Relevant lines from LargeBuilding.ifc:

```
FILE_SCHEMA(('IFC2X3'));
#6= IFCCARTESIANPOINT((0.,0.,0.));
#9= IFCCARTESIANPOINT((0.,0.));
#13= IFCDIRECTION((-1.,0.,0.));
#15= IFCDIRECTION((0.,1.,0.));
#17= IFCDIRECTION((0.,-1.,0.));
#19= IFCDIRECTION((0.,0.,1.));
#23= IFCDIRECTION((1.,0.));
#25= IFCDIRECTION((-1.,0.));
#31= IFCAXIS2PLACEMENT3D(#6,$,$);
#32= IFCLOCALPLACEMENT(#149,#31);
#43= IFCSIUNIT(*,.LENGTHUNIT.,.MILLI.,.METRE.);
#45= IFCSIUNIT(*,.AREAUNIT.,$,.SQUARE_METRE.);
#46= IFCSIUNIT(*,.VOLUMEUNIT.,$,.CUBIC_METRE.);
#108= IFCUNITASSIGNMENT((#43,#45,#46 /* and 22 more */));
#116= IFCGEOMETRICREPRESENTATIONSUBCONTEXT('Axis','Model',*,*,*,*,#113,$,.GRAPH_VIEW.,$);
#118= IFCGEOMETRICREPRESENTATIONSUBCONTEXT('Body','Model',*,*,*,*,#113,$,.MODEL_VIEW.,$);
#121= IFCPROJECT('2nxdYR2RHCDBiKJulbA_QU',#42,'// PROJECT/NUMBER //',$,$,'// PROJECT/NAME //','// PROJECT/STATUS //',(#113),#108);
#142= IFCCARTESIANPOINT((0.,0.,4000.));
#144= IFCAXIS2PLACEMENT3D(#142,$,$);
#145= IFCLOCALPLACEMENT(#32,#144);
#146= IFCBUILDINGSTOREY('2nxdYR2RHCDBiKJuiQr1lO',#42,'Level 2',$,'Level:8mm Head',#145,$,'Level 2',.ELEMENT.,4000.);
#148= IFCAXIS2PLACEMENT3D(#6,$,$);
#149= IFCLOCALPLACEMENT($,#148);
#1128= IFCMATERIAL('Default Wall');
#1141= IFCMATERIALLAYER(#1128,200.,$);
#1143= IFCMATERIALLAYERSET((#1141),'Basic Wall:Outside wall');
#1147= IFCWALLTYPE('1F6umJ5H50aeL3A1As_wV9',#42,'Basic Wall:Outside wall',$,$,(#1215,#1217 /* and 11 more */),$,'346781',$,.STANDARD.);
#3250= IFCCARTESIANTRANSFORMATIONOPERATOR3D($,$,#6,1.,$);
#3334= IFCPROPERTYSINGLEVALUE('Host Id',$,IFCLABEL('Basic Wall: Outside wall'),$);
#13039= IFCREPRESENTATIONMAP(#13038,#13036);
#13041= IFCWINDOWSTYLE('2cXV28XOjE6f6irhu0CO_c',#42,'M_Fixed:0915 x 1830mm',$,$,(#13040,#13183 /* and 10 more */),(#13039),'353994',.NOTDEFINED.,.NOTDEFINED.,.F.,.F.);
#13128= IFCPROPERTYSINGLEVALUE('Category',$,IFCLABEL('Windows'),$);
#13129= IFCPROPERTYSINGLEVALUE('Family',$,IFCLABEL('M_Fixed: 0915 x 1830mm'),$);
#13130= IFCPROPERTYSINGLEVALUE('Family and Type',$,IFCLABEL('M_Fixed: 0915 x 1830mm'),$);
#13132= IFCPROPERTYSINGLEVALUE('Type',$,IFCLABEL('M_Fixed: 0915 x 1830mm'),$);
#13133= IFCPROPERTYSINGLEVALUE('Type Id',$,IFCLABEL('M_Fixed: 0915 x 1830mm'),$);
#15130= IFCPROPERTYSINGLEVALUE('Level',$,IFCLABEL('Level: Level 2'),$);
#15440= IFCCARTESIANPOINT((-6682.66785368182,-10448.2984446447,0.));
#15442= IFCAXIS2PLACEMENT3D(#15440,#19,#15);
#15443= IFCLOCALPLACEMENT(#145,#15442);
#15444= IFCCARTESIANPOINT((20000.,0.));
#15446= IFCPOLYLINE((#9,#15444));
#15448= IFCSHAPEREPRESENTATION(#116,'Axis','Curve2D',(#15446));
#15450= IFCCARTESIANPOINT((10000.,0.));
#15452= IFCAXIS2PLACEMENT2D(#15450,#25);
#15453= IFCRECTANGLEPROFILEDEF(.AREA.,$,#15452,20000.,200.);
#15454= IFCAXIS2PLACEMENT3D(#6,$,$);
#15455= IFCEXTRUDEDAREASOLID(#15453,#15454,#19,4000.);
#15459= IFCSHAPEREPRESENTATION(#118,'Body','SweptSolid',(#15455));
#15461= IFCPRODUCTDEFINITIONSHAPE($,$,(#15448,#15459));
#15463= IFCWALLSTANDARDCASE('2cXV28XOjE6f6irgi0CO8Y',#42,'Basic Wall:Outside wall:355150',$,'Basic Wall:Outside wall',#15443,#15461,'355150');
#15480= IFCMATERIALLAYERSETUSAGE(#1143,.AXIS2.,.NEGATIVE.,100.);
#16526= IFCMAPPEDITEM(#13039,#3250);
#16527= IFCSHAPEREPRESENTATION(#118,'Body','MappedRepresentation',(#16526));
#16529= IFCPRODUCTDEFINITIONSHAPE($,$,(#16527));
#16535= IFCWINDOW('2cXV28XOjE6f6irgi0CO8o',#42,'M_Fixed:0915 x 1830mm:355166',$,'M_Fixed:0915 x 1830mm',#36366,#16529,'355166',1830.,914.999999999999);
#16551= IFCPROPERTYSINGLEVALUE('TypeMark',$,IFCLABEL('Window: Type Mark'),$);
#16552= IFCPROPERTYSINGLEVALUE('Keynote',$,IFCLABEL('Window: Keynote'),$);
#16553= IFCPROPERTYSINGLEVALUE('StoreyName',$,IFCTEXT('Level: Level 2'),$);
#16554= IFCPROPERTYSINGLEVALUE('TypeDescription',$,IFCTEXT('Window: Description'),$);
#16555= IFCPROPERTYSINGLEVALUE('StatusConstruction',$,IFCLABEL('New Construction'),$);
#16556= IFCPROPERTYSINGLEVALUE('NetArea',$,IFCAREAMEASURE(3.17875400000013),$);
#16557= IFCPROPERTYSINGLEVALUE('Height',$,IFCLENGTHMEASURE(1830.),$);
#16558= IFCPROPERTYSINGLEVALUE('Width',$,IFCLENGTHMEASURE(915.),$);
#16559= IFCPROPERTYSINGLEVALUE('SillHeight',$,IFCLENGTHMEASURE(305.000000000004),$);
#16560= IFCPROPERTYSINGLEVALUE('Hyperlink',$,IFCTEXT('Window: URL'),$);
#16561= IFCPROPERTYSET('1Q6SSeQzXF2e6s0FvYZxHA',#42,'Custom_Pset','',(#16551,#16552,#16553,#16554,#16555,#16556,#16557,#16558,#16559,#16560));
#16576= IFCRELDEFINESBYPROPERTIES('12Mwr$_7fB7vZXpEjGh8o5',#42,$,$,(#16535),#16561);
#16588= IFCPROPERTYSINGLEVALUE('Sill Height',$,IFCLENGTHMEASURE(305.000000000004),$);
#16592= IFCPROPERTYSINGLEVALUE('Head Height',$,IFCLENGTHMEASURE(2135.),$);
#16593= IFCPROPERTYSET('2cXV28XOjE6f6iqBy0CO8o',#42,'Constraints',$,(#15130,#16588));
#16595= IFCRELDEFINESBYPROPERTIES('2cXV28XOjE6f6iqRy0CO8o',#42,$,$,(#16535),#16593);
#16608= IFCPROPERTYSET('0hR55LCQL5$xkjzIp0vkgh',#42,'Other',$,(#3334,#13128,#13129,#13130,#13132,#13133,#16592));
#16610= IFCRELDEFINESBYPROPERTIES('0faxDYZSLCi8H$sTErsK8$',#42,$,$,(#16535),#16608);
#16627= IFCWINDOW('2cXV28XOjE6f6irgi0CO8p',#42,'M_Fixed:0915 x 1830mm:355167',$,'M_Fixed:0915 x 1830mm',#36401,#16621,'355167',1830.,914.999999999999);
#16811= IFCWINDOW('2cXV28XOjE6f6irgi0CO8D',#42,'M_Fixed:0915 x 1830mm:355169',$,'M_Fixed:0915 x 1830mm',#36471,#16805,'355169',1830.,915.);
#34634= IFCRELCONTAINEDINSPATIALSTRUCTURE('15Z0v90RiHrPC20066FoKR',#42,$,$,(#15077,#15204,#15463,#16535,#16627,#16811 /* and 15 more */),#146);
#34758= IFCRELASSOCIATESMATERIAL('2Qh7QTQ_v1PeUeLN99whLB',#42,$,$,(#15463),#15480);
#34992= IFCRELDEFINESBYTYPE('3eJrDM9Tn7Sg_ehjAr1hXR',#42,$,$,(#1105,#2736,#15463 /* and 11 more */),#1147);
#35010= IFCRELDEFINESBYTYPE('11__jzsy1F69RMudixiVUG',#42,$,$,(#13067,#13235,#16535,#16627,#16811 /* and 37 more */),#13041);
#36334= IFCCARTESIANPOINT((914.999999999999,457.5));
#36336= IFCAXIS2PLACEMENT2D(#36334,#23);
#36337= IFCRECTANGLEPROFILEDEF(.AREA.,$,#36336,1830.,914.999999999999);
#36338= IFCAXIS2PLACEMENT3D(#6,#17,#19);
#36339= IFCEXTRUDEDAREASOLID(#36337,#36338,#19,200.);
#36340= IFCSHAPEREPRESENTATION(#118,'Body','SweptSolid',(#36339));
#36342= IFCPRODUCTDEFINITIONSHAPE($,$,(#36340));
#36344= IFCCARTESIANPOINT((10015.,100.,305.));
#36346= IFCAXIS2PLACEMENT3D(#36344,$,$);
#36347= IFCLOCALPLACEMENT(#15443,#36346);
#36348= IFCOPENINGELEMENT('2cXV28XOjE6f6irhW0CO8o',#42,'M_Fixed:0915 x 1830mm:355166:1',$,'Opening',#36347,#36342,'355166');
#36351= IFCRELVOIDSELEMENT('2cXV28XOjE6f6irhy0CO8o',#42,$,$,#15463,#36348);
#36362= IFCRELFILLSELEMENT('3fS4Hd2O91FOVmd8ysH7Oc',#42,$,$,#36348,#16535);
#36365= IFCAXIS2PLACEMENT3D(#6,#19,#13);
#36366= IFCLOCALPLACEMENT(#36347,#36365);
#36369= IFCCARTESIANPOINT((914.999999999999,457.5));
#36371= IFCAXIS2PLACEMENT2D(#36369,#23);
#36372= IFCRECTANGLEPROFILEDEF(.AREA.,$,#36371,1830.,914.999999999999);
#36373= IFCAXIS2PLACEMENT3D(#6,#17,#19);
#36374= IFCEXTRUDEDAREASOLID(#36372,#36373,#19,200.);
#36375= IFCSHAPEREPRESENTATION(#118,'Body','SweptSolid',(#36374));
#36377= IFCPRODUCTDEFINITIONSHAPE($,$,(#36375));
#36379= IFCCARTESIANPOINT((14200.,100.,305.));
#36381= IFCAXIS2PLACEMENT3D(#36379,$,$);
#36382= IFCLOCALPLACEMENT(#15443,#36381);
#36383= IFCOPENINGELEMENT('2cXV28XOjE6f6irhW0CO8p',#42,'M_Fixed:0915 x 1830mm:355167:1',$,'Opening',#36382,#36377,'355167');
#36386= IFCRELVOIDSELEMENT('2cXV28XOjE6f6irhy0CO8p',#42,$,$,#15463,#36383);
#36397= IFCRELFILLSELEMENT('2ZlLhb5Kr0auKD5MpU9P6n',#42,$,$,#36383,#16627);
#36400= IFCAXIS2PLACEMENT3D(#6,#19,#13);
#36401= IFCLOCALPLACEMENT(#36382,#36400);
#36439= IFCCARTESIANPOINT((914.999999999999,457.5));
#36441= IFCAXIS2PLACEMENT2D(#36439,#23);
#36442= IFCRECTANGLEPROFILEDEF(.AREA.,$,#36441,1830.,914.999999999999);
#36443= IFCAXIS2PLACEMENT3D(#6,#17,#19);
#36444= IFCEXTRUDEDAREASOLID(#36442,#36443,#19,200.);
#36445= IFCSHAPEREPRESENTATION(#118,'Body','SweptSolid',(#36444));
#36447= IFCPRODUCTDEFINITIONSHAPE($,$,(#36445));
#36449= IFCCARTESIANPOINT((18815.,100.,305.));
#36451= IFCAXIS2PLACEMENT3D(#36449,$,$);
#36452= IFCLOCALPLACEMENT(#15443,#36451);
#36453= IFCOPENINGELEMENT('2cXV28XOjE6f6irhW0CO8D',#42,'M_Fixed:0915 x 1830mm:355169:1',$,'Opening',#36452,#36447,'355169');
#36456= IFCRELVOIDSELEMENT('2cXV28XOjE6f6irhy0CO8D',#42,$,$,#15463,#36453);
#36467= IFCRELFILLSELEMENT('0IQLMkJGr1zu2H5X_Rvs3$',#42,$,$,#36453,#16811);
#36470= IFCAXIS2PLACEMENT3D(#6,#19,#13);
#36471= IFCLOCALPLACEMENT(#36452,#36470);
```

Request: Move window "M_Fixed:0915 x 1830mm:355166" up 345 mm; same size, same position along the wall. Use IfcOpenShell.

```python
import numpy as np
import ifcopenshell
import ifcopenshell.api.geometry
import ifcopenshell.api.pset
import ifcopenshell.util.element
import ifcopenshell.util.placement
import ifcopenshell.util.unit

model = ifcopenshell.open("LargeBuilding.ifc")
unit_scale = ifcopenshell.util.unit.calculate_unit_scale(model)

window = model.by_guid("2cXV28XOjE6f6irgi0CO8o")
opening = window.FillsVoids[0].RelatingOpeningElement
dz = 345.0

shift = np.array([0.0, 0.0, dz])
# The window is placed relative to its opening, so it follows when the opening moves.
matrix = ifcopenshell.util.placement.get_local_placement(opening.ObjectPlacement)
matrix[:3, 3] += shift
ifcopenshell.api.geometry.edit_object_placement(
    model, product=opening, matrix=matrix, is_si=False, should_transform_children=True
)

# Keep the stored heights in step.
pset = model.by_id(ifcopenshell.util.element.get_pset(window, "Custom_Pset", should_inherit=False)["id"])
ifcopenshell.api.pset.edit_pset(model, pset=pset, properties={
    "SillHeight": model.create_entity("IfcLengthMeasure", ifcopenshell.util.element.get_pset(window, "Constraints", "Sill Height") + dz),
})
pset = model.by_id(ifcopenshell.util.element.get_pset(window, "Constraints", should_inherit=False)["id"])
ifcopenshell.api.pset.edit_pset(model, pset=pset, properties={
    "Sill Height": model.create_entity("IfcLengthMeasure", ifcopenshell.util.element.get_pset(window, "Constraints", "Sill Height") + dz),
})
pset = model.by_id(ifcopenshell.util.element.get_pset(window, "Other", should_inherit=False)["id"])
ifcopenshell.api.pset.edit_pset(model, pset=pset, properties={
    "Head Height": model.create_entity("IfcLengthMeasure", ifcopenshell.util.element.get_pset(window, "Other", "Head Height") + dz),
})

print(f"moved by {dz * unit_scale:+.3f} m")

model.write("LargeBuilding_rev.ifc")
```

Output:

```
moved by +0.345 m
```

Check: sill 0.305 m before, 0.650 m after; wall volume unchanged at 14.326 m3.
